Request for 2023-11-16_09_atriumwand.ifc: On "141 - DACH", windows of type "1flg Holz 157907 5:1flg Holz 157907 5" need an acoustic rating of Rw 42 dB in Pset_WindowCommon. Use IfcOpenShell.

First a look at what the model holds.

```python
import ifcopenshell
import ifcopenshell.util.element

model = ifcopenshell.open("2023-11-16_09_atriumwand.ifc")
print(model.schema)
storey = next(s for s in model.by_type("IfcBuildingStorey") if s.Name == "141 - DACH")
windows = [e for e in ifcopenshell.util.element.get_decomposition(storey) if e.is_a("IfcWindow")]
seen = {}
for e in windows:
    element_type = ifcopenshell.util.element.get_type(e)
    key = (element_type.Name if element_type != e and element_type else None, ifcopenshell.util.element.get_pset(e, "Pset_WindowCommon", "AcousticRating"))
    seen[key] = seen.get(key, 0) + 1
for (name, value), count in sorted(seen.items(), key=str):
    print(count, "x", name, "|", value)
```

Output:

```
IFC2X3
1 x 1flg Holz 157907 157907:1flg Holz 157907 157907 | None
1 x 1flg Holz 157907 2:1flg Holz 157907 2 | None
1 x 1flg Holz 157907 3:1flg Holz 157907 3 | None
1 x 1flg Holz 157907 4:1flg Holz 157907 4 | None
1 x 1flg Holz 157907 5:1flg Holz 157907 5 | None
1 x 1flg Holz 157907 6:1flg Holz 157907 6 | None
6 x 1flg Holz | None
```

```python
import ifcopenshell
import ifcopenshell.api.pset
import ifcopenshell.util.element

model = ifcopenshell.open("2023-11-16_09_atriumwand.ifc")

storey = next(s for s in model.by_type("IfcBuildingStorey") if s.Name == "141 - DACH")
windows = [e for e in ifcopenshell.util.element.get_decomposition(storey) if e.is_a("IfcWindow")]

count = 0
for e in windows:
    element_type = ifcopenshell.util.element.get_type(e)
    if element_type in (None, e) or element_type.Name != "1flg Holz 157907 5:1flg Holz 157907 5":
        continue
    # add_pset returns the element's existing set when there is one.
    pset = ifcopenshell.api.pset.add_pset(model, product=e, name="Pset_WindowCommon")
    ifcopenshell.api.pset.edit_pset(model, pset=pset, properties={"AcousticRating": "Rw 42 dB"})
    count += 1

print(count, "windows updated")

model.write("2023-11-16_09_atriumwand-out.ifc")
```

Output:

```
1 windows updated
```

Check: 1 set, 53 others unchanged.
